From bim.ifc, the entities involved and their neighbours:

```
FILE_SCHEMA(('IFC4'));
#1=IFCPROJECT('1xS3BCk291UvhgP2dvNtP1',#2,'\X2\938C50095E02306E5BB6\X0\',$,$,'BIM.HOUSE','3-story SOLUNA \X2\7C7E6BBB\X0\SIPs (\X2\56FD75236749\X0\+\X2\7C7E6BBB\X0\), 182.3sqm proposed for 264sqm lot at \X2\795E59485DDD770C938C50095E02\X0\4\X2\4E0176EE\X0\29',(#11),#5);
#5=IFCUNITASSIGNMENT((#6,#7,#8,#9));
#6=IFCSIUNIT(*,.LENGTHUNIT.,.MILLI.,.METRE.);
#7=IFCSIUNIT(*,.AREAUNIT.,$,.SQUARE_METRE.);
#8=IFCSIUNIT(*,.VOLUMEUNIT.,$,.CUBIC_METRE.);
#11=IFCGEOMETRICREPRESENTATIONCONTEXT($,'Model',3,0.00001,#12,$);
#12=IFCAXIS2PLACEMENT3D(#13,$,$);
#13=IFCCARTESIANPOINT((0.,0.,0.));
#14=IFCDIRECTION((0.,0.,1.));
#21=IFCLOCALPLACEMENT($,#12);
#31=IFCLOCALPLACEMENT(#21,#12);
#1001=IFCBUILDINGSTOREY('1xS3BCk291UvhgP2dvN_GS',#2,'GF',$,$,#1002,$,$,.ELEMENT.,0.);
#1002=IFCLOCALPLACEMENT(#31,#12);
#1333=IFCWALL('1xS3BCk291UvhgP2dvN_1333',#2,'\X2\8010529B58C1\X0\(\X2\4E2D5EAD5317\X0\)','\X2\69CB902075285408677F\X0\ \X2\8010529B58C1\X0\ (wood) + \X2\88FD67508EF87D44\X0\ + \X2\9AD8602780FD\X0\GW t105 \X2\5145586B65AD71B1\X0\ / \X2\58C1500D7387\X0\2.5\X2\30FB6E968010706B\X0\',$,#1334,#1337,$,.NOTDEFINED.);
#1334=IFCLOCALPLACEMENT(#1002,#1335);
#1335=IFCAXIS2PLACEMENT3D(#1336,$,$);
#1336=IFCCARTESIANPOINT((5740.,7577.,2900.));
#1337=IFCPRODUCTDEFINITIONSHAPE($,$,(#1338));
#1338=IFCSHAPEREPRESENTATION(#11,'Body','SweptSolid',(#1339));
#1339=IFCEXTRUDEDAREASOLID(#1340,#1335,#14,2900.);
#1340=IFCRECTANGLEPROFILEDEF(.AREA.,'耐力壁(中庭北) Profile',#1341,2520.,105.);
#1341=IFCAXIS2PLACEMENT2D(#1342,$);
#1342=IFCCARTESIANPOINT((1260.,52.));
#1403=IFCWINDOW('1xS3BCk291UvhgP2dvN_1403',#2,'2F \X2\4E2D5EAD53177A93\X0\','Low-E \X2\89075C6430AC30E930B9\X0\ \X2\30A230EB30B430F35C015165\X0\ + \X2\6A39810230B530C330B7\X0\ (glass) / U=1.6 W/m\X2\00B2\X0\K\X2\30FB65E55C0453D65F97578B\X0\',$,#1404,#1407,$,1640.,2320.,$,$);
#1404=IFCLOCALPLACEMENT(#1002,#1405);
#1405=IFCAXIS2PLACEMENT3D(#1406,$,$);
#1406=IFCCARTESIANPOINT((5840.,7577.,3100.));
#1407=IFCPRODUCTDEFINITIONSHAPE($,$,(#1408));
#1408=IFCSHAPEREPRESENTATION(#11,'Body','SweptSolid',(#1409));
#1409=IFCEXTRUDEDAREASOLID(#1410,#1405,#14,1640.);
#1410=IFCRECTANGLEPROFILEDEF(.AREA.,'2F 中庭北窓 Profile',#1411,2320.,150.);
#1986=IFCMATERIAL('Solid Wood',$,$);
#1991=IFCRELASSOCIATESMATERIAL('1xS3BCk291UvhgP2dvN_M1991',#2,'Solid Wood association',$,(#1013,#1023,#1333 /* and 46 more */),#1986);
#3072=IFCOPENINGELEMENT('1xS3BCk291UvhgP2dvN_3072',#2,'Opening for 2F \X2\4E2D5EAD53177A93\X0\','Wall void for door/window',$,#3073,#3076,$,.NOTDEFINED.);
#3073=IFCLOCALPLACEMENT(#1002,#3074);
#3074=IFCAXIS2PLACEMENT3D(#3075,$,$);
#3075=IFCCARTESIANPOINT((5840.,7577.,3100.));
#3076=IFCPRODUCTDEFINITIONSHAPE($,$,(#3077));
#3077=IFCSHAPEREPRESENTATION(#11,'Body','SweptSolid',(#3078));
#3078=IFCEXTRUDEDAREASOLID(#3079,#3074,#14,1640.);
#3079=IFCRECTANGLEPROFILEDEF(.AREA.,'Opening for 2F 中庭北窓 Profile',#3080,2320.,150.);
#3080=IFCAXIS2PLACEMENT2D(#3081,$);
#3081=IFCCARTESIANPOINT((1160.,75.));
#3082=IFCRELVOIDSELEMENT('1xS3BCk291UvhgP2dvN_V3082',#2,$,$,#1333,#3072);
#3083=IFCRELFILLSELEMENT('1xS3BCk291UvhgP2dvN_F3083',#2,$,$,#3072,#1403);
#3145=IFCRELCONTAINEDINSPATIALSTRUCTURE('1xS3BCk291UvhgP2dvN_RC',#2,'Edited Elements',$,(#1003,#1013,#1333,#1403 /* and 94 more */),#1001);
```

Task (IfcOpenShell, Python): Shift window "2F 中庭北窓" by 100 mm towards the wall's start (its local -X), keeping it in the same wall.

```python
import ifcopenshell
import ifcopenshell.api.geometry
import ifcopenshell.util.placement
import ifcopenshell.util.unit

model = ifcopenshell.open("bim.ifc")
unit_scale = ifcopenshell.util.unit.calculate_unit_scale(model)

window = model.by_guid("1xS3BCk291UvhgP2dvN_1403")
opening = window.FillsVoids[0].RelatingOpeningElement
wall = opening.VoidsElements[0].RelatingBuildingElement

wall_matrix = ifcopenshell.util.placement.get_local_placement(wall.ObjectPlacement)
shift = wall_matrix[:3, 0] * -0.1 / unit_scale
before = ifcopenshell.util.placement.get_local_placement(window.ObjectPlacement)[:3, 3].copy()

# The window is not placed relative to its opening, so move both.
for product in (opening, window):
    matrix = ifcopenshell.util.placement.get_local_placement(product.ObjectPlacement)
    matrix[:3, 3] += shift
    ifcopenshell.api.geometry.edit_object_placement(model, product=product, matrix=matrix, is_si=False)

after = ifcopenshell.util.placement.get_local_placement(window.ObjectPlacement)[:3, 3]
print("window moved by", (after - before).round(3) + 0.0)

model.write("bim-out.ifc")
```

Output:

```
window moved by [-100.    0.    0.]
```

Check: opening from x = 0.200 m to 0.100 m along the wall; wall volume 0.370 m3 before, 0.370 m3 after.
